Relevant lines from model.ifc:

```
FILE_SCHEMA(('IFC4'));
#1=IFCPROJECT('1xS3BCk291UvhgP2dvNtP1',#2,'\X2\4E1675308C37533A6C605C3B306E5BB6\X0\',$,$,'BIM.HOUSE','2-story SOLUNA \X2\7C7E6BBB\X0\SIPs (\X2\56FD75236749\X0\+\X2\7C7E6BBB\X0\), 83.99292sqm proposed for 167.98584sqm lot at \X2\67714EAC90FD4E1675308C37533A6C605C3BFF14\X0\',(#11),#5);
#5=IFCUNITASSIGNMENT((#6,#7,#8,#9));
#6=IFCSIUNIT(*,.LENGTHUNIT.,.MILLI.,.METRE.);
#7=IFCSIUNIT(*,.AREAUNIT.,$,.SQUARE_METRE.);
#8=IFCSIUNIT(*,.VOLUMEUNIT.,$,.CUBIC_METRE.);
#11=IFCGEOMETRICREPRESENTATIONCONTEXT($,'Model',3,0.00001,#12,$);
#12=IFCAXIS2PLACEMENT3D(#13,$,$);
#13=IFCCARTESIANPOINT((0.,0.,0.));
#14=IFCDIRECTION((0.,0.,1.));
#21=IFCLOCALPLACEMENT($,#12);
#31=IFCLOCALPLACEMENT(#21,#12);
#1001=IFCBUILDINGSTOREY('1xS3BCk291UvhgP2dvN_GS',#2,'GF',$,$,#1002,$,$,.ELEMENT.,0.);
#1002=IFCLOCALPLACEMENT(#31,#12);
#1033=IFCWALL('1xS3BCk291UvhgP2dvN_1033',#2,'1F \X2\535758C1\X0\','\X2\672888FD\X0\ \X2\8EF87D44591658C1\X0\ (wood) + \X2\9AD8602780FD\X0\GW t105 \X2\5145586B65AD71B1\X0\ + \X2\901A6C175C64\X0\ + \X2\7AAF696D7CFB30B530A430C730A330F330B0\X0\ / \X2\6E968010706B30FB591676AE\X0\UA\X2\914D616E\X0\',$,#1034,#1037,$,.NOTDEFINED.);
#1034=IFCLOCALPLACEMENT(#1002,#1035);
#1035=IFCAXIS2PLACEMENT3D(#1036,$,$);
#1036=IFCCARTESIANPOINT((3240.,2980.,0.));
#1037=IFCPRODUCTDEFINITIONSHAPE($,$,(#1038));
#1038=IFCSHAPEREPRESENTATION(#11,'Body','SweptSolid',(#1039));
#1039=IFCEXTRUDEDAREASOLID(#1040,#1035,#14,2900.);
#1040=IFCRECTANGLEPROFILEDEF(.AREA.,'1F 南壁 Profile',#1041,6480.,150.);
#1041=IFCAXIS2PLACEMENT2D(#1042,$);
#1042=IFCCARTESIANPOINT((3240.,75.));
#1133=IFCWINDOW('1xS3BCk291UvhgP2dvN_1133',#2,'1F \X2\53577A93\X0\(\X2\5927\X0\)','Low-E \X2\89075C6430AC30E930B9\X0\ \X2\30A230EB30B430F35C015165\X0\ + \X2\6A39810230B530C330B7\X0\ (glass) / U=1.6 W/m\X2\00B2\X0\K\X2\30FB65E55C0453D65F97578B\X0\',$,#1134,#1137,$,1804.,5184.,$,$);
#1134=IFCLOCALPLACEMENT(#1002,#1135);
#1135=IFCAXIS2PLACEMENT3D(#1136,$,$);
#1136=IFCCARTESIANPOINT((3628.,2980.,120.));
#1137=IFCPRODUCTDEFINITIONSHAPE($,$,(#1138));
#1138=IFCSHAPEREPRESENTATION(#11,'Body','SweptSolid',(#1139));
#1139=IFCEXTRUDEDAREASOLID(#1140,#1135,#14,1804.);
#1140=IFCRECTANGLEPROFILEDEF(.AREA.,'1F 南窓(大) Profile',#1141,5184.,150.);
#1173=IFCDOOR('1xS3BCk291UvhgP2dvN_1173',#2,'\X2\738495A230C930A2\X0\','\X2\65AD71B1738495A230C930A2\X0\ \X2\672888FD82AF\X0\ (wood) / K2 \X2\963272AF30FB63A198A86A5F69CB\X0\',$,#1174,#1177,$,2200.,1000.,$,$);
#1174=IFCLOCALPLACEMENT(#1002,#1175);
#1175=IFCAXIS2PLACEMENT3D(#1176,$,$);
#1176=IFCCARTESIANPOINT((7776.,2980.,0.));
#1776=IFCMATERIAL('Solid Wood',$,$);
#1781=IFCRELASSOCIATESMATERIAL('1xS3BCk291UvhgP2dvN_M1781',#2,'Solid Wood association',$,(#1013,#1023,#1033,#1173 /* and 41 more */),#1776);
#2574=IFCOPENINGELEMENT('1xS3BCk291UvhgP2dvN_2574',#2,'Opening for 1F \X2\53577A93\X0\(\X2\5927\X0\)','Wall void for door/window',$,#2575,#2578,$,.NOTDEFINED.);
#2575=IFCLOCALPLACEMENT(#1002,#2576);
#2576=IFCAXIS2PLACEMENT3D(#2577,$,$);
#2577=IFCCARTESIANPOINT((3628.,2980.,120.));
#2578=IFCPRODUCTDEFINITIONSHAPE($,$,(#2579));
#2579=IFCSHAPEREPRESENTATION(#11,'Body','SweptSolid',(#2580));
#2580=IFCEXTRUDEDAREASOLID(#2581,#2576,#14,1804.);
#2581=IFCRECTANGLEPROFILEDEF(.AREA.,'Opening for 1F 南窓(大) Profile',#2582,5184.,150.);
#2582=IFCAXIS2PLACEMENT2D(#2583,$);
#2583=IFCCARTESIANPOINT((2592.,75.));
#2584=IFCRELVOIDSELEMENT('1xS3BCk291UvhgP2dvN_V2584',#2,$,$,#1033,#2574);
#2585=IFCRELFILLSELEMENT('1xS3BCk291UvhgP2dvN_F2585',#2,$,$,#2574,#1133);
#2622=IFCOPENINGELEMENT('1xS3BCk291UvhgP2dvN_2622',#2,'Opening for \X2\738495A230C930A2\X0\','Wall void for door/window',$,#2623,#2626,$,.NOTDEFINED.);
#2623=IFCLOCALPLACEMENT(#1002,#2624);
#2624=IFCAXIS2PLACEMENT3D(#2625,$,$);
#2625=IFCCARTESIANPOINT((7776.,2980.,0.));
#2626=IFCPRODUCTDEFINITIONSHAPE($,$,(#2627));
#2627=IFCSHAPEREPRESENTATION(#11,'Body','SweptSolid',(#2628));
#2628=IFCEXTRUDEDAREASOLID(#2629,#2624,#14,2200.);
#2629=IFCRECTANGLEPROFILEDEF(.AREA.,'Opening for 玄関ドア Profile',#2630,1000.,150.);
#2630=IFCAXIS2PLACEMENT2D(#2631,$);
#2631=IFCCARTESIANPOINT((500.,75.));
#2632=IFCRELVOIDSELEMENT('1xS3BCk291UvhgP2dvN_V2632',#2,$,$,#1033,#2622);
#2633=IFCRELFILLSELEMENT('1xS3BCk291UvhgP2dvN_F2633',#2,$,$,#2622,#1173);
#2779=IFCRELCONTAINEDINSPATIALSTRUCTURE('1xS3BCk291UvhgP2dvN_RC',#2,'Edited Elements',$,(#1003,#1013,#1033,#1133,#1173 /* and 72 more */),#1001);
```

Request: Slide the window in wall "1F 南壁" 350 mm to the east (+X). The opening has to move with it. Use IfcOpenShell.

```python
import ifcopenshell
import ifcopenshell.api.geometry
import ifcopenshell.util.placement

model = ifcopenshell.open("model.ifc")

window = model.by_id(1133)
opening = window.FillsVoids[0].RelatingOpeningElement
wall = opening.VoidsElements[0].RelatingBuildingElement

wall_matrix = ifcopenshell.util.placement.get_local_placement(wall.ObjectPlacement)
shift = wall_matrix[:3, 0] * 350.0
before = ifcopenshell.util.placement.get_local_placement(window.ObjectPlacement)[:3, 3].copy()

# The window is not placed relative to its opening, so move both.
for product in (opening, window):
    matrix = ifcopenshell.util.placement.get_local_placement(product.ObjectPlacement)
    matrix[:3, 3] += shift
    ifcopenshell.api.geometry.edit_object_placement(model, product=product, matrix=matrix, is_si=False)

after = ifcopenshell.util.placement.get_local_placement(window.ObjectPlacement)[:3, 3]
print("window moved by", (after - before).round(3) + 0.0)

model.write("model_rev.ifc")
```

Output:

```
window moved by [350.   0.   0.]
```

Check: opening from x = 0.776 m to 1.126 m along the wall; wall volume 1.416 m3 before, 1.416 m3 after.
